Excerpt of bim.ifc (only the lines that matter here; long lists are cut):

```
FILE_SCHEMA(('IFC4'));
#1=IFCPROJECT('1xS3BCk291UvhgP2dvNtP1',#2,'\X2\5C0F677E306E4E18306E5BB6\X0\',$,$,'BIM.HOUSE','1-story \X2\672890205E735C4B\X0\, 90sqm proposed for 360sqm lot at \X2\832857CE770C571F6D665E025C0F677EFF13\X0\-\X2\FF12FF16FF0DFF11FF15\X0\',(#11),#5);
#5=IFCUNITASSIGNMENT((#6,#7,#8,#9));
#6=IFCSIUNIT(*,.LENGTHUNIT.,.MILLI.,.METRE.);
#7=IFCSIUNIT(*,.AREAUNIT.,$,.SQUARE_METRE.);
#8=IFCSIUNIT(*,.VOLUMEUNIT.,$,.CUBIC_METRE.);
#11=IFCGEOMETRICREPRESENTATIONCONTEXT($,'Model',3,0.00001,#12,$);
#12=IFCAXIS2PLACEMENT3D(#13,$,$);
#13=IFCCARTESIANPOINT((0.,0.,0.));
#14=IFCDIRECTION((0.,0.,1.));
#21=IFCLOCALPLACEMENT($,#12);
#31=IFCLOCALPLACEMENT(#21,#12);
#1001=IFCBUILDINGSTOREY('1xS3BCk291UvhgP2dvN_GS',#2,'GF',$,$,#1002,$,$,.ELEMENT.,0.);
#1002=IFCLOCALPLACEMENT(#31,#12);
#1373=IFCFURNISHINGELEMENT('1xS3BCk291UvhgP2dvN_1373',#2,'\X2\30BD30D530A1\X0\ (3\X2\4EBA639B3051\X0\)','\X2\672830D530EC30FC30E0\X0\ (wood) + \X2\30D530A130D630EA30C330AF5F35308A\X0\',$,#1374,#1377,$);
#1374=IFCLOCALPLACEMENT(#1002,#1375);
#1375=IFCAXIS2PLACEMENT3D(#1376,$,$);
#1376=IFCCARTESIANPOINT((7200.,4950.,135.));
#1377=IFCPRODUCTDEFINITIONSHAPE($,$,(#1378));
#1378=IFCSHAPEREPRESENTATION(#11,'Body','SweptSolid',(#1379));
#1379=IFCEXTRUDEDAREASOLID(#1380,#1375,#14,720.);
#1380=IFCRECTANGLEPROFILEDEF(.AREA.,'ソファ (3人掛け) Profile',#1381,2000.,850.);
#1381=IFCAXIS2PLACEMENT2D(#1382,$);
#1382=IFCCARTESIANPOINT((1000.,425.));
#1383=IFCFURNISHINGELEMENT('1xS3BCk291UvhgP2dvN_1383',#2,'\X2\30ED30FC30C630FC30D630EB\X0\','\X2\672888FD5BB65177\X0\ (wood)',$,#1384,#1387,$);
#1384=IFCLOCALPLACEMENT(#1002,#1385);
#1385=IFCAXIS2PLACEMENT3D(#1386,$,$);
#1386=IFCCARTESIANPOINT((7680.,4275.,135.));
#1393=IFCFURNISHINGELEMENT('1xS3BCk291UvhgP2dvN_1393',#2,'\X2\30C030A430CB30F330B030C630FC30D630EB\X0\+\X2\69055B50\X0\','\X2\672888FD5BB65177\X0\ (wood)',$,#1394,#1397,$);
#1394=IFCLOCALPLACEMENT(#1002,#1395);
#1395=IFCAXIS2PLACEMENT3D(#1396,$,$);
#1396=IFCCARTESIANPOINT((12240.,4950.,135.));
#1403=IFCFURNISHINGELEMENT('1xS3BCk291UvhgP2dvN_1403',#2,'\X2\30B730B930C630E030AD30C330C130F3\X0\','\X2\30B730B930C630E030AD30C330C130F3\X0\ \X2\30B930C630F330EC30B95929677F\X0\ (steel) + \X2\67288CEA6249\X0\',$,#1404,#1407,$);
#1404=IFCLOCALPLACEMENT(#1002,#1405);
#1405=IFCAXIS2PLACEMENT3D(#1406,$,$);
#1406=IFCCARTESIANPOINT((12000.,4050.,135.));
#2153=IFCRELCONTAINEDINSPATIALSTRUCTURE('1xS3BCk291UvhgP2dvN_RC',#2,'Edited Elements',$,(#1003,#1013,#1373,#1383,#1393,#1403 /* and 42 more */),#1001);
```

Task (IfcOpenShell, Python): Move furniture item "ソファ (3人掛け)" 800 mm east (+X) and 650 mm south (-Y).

```python
import ifcopenshell
import ifcopenshell.api.geometry
import ifcopenshell.util.placement

model = ifcopenshell.open("bim.ifc")

item = model.by_guid("1xS3BCk291UvhgP2dvN_1373")
matrix = ifcopenshell.util.placement.get_local_placement(item.ObjectPlacement)
matrix[0, 3] += 800.0
matrix[1, 3] -= 650.0
ifcopenshell.api.geometry.edit_object_placement(model, product=item, matrix=matrix, is_si=False)

print(ifcopenshell.util.placement.get_local_placement(item.ObjectPlacement).round(3) + 0.0)

model.write("bim_v2.ifc")
```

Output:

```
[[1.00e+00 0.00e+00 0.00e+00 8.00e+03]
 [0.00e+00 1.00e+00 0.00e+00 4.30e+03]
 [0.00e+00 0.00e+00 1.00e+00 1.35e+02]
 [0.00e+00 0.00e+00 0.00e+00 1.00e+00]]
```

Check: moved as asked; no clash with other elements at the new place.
